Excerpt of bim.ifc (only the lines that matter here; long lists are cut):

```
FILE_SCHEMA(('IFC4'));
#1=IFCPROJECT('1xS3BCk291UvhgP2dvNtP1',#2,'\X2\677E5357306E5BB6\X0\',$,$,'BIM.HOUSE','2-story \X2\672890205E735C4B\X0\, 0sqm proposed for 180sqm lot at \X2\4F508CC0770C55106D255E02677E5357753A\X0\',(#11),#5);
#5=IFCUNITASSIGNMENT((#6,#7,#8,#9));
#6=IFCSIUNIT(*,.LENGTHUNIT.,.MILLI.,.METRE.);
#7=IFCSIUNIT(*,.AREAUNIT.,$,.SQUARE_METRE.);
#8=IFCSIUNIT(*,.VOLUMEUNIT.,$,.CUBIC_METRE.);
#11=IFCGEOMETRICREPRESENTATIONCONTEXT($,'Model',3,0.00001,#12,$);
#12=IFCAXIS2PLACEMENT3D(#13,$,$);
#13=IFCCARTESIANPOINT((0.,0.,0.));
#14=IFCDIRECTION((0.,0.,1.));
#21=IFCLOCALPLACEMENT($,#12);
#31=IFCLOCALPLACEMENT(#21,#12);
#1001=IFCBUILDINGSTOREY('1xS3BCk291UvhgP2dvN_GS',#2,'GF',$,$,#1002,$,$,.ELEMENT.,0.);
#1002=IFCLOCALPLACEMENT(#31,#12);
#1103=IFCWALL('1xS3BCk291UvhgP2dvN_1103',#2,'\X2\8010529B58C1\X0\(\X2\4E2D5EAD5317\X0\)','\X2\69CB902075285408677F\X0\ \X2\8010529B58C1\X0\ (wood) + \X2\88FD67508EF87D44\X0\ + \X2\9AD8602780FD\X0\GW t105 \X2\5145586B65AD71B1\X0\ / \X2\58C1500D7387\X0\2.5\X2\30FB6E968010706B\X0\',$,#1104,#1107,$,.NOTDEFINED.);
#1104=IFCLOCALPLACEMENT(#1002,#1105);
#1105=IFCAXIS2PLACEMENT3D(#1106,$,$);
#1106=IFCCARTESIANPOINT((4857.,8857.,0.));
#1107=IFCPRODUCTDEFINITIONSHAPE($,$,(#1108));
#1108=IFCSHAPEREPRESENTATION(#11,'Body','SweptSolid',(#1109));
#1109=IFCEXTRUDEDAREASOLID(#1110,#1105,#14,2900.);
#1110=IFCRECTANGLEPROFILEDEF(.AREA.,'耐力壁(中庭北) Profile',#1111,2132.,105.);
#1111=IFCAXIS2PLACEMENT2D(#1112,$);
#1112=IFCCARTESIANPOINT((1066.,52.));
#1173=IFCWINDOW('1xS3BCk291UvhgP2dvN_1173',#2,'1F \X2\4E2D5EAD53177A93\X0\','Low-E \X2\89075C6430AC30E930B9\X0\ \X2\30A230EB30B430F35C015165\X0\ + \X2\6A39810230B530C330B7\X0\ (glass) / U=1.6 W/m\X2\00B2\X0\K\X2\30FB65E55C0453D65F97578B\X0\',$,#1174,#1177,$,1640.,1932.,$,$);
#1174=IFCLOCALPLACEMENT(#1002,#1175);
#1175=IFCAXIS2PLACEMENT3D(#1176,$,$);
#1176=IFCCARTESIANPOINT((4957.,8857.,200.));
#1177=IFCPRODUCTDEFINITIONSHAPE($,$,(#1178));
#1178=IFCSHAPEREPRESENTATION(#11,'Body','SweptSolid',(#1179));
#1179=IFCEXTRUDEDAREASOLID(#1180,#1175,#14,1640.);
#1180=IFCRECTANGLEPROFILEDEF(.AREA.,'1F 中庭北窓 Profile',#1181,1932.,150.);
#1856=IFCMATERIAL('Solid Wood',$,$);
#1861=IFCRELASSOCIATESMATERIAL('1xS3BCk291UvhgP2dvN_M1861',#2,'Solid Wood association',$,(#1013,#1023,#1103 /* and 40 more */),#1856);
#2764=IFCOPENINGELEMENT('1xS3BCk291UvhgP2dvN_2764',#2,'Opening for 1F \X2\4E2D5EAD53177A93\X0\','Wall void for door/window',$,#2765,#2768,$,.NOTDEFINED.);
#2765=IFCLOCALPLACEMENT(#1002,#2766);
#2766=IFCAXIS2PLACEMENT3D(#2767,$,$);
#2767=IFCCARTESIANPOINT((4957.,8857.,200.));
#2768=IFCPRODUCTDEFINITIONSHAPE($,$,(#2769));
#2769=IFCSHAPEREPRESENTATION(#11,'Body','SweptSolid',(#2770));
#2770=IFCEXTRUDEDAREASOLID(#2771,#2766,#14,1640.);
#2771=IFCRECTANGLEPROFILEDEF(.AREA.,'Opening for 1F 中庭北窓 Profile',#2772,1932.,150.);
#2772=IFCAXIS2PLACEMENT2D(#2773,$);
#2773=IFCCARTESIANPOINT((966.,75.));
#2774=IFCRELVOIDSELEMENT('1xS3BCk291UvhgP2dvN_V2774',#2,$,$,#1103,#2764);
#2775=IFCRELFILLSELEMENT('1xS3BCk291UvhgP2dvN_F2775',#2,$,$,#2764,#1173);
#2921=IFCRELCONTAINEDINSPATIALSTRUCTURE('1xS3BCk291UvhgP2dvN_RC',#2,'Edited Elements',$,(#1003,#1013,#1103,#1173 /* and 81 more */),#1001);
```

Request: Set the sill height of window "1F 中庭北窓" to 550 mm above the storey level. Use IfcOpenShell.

```python
import numpy as np
import ifcopenshell
import ifcopenshell.api.geometry
import ifcopenshell.geom
import ifcopenshell.util.element
import ifcopenshell.util.placement
import ifcopenshell.util.shape
import ifcopenshell.util.unit

model = ifcopenshell.open("bim.ifc")
unit_scale = ifcopenshell.util.unit.calculate_unit_scale(model)

window = model.by_id(1173)
opening = window.FillsVoids[0].RelatingOpeningElement
storey = ifcopenshell.util.element.get_container(window, ifc_class="IfcBuildingStorey")
level = ifcopenshell.util.placement.get_local_placement(storey.ObjectPlacement)[2, 3]

# The opening's origin need not be at the sill, so measure its lowest point.
shape = ifcopenshell.geom.create_shape(ifcopenshell.geom.settings(), opening)
bottom = ifcopenshell.util.shape.get_shape_bottom_elevation(shape, shape.geometry) / unit_scale
dz = level + 0.55 / unit_scale - bottom

shift = np.array([0.0, 0.0, dz])
# The window is not placed relative to its opening, so move both.
for product in (opening, window):
    matrix = ifcopenshell.util.placement.get_local_placement(product.ObjectPlacement)
    matrix[:3, 3] += shift
    ifcopenshell.api.geometry.edit_object_placement(model, product=product, matrix=matrix, is_si=False)

print(f"moved by {dz * unit_scale:+.3f} m")

model.write("bim_v2.ifc")
```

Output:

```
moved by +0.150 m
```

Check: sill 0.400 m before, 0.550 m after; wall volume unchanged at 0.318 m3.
